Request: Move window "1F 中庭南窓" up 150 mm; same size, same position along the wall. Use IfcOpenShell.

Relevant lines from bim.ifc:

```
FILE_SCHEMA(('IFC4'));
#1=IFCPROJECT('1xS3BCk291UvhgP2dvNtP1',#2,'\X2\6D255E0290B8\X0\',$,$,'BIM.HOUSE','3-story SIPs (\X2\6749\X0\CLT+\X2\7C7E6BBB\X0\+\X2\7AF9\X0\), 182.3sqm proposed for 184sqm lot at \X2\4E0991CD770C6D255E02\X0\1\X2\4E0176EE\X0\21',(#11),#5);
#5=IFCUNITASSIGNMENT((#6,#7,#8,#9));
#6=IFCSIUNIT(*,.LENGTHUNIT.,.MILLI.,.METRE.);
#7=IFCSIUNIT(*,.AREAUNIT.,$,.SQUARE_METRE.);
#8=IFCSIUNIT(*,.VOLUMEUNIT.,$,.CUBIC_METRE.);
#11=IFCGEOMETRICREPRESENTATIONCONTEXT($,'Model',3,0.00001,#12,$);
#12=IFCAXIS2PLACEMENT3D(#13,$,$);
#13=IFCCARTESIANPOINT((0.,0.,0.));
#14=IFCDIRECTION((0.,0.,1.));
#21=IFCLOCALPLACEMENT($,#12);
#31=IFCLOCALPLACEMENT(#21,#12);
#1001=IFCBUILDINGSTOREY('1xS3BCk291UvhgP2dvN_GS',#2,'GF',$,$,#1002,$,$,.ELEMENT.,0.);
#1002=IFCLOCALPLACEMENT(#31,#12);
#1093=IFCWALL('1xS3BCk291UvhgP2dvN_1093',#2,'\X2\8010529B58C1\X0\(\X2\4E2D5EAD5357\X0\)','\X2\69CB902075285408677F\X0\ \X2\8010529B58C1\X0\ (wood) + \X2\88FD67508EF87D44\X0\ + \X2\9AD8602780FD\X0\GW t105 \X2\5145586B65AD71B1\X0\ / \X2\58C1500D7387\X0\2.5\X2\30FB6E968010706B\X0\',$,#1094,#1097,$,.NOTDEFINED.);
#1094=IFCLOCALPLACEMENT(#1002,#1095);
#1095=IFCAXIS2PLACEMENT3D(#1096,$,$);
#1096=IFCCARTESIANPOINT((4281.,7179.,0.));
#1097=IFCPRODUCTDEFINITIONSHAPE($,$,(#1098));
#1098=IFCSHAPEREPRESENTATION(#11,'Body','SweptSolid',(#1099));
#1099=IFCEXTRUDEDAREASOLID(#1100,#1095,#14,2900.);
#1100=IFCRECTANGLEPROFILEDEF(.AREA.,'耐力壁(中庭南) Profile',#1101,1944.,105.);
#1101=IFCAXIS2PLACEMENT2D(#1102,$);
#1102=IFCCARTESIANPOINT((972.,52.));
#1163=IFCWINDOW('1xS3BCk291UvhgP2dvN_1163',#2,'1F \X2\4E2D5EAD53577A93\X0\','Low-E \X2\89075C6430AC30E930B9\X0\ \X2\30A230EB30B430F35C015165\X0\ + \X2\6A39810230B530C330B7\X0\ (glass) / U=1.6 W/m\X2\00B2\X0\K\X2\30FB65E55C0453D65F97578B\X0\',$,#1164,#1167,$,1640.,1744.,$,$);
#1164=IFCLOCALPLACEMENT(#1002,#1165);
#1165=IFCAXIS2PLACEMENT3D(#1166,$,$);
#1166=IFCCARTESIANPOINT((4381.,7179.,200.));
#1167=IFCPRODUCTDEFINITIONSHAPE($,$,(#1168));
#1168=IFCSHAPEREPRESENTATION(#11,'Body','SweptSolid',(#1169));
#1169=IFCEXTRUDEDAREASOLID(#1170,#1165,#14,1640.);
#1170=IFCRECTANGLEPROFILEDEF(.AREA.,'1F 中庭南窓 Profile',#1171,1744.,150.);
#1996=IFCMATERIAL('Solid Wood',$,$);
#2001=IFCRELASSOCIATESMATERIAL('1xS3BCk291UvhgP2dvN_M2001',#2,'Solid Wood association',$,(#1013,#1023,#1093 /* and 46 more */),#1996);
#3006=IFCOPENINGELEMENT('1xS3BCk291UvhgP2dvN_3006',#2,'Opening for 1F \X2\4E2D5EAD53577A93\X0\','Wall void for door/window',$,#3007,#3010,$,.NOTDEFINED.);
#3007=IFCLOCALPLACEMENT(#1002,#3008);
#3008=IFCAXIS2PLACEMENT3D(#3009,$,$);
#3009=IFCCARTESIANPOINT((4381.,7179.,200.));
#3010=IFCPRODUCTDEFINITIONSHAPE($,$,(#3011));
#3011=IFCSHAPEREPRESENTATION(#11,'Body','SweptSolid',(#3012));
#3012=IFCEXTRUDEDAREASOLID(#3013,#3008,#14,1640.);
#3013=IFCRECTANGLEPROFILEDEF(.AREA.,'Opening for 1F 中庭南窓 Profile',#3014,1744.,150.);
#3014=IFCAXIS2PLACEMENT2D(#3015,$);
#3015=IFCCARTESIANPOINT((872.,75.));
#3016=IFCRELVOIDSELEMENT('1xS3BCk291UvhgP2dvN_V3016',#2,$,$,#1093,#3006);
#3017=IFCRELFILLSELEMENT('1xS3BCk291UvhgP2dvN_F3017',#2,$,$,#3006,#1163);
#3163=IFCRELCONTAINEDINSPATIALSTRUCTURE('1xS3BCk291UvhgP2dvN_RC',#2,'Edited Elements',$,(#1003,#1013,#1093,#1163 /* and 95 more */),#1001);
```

```python
import numpy as np
import ifcopenshell
import ifcopenshell.api.geometry
import ifcopenshell.util.placement
import ifcopenshell.util.unit

model = ifcopenshell.open("bim.ifc")
unit_scale = ifcopenshell.util.unit.calculate_unit_scale(model)

window = model.by_guid("1xS3BCk291UvhgP2dvN_1163")
opening = window.FillsVoids[0].RelatingOpeningElement
dz = 0.15 / unit_scale

shift = np.array([0.0, 0.0, dz])
# The window is not placed relative to its opening, so move both.
for product in (opening, window):
    matrix = ifcopenshell.util.placement.get_local_placement(product.ObjectPlacement)
    matrix[:3, 3] += shift
    ifcopenshell.api.geometry.edit_object_placement(model, product=product, matrix=matrix, is_si=False)

print(f"moved by {dz * unit_scale:+.3f} m")

model.write("bim-out.ifc")
```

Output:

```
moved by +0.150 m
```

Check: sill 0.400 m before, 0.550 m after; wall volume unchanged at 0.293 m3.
